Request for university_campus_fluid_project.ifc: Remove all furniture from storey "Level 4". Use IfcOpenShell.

First a look at what the model holds.

```python
import ifcopenshell
import ifcopenshell.util.element

model = ifcopenshell.open("university_campus_fluid_project.ifc")
print(model.schema)
storey = next(s for s in model.by_type("IfcBuildingStorey") if s.Name == "Level 4")
furniture = [e for e in ifcopenshell.util.element.get_decomposition(storey) if e.is_a("IfcFurnishingElement")]
seen = {}
for e in furniture:
    element_type = ifcopenshell.util.element.get_type(e)
    name = element_type.Name if element_type not in (None, e) else None
    seen[name] = seen.get(name, 0) + 1
for name, count in sorted(seen.items(), key=str):
    print(count, "x", name)
```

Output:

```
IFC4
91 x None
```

```python
import ifcopenshell
import ifcopenshell.api.root
import ifcopenshell.util.element

model = ifcopenshell.open("university_campus_fluid_project.ifc")

storey = next(s for s in model.by_type("IfcBuildingStorey") if s.Name == "Level 4")
furniture = [e for e in ifcopenshell.util.element.get_decomposition(storey) if e.is_a("IfcFurnishingElement")]

for e in furniture:
    ifcopenshell.api.root.remove_product(model, product=e)
print(len(furniture), "removed")

model.write("university_campus_fluid_project_v2.ifc")
```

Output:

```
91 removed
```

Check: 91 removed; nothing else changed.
